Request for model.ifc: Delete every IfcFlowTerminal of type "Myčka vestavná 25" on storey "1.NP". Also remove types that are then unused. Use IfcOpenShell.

First a look at what the model holds.

```python
import ifcopenshell
import ifcopenshell.util.element

model = ifcopenshell.open("model.ifc")
print(model.schema)
storey = next(s for s in model.by_type("IfcBuildingStorey") if s.Name == "1.NP")
terminals = [e for e in ifcopenshell.util.element.get_decomposition(storey) if e.is_a("IfcFlowTerminal")]
seen = {}
for e in terminals:
    element_type = ifcopenshell.util.element.get_type(e)
    name = element_type.Name if element_type not in (None, e) else None
    seen[name] = seen.get(name, 0) + 1
for name, count in sorted(seen.items(), key=str):
    print(count, "x", name)
```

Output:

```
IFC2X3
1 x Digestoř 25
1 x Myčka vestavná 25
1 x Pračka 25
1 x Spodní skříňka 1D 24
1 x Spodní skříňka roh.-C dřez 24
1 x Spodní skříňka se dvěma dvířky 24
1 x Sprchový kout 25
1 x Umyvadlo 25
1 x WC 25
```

```python
import ifcopenshell
import ifcopenshell.api.root
import ifcopenshell.util.element

model = ifcopenshell.open("model.ifc")

storey = next(s for s in model.by_type("IfcBuildingStorey") if s.Name == "1.NP")
terminals = [e for e in ifcopenshell.util.element.get_decomposition(storey) if e.is_a("IfcFlowTerminal")]
targets = [e for e in terminals if (t := ifcopenshell.util.element.get_type(e)) not in (None, e) and t.Name == "Myčka vestavná 25"]
types = {ifcopenshell.util.element.get_type(e) for e in targets} - {None, *targets}

for e in targets:
    ifcopenshell.api.root.remove_product(model, product=e)
print(len(targets), "removed")

unused = [t for t in types if not ifcopenshell.util.element.get_types(t)]
for t in unused:
    ifcopenshell.api.root.remove_product(model, product=t)
print(len(unused), "unused types removed")

model.write("model_edited.ifc")
```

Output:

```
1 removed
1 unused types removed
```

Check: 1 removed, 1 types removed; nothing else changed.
